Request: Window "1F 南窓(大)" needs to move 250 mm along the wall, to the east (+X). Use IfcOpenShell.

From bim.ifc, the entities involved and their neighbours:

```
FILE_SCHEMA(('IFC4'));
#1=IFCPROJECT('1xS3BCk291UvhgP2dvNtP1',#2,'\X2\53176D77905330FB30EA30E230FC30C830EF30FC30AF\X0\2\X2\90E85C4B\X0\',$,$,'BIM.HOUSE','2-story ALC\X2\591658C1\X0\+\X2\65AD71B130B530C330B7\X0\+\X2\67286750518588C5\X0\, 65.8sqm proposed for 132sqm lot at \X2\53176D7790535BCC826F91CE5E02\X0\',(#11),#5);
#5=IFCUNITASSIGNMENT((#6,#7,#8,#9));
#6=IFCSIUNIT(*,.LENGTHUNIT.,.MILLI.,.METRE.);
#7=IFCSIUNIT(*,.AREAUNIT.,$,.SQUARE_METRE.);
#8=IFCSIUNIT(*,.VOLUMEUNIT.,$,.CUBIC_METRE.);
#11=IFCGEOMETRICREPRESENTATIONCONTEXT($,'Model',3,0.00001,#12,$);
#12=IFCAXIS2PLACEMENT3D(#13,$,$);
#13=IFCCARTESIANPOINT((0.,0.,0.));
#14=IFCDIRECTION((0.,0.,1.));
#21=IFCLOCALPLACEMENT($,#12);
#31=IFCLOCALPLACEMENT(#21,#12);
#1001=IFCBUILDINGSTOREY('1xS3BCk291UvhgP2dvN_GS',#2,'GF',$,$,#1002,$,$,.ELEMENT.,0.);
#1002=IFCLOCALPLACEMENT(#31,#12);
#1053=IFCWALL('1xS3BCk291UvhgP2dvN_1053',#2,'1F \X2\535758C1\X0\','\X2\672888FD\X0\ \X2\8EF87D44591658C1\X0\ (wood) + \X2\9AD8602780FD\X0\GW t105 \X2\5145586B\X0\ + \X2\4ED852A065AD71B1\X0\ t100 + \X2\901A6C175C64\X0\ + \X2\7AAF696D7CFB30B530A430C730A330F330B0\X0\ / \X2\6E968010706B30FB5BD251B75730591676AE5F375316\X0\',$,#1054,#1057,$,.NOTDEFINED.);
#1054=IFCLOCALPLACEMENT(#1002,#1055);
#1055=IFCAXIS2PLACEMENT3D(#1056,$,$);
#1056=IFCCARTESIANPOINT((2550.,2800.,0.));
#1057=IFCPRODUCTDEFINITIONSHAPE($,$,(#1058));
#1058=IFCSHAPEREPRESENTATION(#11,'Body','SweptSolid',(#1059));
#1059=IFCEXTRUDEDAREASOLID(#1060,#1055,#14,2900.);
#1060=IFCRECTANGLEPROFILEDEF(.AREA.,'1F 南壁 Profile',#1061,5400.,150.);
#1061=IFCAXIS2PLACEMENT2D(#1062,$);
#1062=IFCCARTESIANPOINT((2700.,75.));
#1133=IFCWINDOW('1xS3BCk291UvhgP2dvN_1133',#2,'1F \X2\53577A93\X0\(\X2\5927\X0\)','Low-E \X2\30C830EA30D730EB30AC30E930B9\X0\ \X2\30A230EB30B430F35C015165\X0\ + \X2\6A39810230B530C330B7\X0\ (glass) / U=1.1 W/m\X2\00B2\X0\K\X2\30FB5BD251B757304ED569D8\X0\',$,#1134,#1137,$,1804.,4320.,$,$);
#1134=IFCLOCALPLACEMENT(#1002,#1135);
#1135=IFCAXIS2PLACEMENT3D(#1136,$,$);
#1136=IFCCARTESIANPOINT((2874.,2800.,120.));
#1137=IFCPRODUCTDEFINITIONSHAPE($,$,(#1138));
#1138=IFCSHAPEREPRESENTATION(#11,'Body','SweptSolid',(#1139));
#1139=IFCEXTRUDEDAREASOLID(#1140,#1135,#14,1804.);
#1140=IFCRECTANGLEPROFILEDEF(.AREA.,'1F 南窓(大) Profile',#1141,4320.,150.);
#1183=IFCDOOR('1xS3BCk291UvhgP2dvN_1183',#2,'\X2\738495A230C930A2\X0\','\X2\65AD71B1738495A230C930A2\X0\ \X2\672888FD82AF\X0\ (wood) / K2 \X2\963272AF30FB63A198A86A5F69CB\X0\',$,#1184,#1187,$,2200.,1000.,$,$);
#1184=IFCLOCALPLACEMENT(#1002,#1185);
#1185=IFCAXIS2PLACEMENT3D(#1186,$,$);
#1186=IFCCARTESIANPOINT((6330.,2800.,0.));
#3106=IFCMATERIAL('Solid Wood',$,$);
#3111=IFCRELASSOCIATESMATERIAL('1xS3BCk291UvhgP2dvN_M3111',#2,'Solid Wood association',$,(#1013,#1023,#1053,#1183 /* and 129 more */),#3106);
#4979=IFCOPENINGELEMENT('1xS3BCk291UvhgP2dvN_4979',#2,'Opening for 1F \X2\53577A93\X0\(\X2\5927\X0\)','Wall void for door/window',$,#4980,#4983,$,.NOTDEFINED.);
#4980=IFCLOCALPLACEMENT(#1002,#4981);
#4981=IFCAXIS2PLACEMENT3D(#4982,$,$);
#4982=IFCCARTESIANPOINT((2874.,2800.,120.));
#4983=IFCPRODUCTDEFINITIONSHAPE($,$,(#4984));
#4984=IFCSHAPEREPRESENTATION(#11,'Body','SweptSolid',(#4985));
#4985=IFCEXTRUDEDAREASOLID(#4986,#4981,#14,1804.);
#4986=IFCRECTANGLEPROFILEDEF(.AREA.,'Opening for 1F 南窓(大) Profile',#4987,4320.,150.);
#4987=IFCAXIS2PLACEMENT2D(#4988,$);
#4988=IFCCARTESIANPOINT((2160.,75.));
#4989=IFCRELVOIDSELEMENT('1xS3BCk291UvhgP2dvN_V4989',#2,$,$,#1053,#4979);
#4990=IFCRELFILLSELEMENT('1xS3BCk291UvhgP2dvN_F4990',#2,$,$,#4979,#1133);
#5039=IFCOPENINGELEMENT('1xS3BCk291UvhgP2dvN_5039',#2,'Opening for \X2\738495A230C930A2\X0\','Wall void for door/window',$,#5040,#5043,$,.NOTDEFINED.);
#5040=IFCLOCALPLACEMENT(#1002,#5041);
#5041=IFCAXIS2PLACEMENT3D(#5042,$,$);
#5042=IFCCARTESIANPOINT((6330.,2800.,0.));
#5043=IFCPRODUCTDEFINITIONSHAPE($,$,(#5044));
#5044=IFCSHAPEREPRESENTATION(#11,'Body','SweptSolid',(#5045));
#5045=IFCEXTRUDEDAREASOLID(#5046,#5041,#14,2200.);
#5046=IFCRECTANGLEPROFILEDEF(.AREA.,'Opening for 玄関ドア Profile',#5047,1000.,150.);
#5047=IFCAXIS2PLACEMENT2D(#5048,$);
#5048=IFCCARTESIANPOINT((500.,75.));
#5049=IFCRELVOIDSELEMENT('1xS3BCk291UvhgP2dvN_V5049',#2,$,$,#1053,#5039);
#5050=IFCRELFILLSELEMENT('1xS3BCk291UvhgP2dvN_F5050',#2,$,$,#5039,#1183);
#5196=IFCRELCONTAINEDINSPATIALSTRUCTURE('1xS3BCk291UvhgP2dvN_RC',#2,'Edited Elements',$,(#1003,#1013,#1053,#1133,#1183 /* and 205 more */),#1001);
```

```python
import ifcopenshell
import ifcopenshell.api.geometry
import ifcopenshell.util.placement
import ifcopenshell.util.unit

model = ifcopenshell.open("bim.ifc")
unit_scale = ifcopenshell.util.unit.calculate_unit_scale(model)

window = model.by_guid("1xS3BCk291UvhgP2dvN_1133")
opening = window.FillsVoids[0].RelatingOpeningElement
wall = opening.VoidsElements[0].RelatingBuildingElement

wall_matrix = ifcopenshell.util.placement.get_local_placement(wall.ObjectPlacement)
shift = wall_matrix[:3, 0] * 0.25 / unit_scale
before = ifcopenshell.util.placement.get_local_placement(window.ObjectPlacement)[:3, 3].copy()

# The window is not placed relative to its opening, so move both.
for product in (opening, window):
    matrix = ifcopenshell.util.placement.get_local_placement(product.ObjectPlacement)
    matrix[:3, 3] += shift
    ifcopenshell.api.geometry.edit_object_placement(model, product=product, matrix=matrix, is_si=False)

after = ifcopenshell.util.placement.get_local_placement(window.ObjectPlacement)[:3, 3]
print("window moved by", (after - before).round(3) + 0.0)

model.write("bim_v2.ifc")
```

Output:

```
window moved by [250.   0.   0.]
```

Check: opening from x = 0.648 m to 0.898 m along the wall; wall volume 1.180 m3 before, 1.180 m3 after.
